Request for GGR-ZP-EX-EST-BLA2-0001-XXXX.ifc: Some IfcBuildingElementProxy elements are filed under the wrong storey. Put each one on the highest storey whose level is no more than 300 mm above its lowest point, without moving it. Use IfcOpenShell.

First a look at what the model holds.

```python
import ifcopenshell
import ifcopenshell.util.element
import ifcopenshell.util.placement

model = ifcopenshell.open("GGR-ZP-EX-EST-BLA2-0001-XXXX.ifc")
print(model.schema)
for storey in model.by_type("IfcBuildingStorey"):
    level = ifcopenshell.util.placement.get_storey_elevation(storey)
    count = sum(e.is_a("IfcBuildingElementProxy") for e in ifcopenshell.util.element.get_contained(storey))
    print(storey.id(), storey.Name, round(level, 3), count, sep=" | ")
```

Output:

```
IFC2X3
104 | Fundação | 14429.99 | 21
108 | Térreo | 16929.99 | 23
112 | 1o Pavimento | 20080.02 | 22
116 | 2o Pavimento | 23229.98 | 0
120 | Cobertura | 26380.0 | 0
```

```python
import ifcopenshell
import ifcopenshell.api.spatial
import ifcopenshell.geom
import ifcopenshell.util.element
import ifcopenshell.util.placement
import ifcopenshell.util.shape
import ifcopenshell.util.unit

model = ifcopenshell.open("GGR-ZP-EX-EST-BLA2-0001-XXXX.ifc")
unit_scale = ifcopenshell.util.unit.calculate_unit_scale(model)
settings = ifcopenshell.geom.settings()

levels = sorted(
    ((ifcopenshell.util.placement.get_storey_elevation(s) * unit_scale, s) for s in model.by_type("IfcBuildingStorey")),
    key=lambda pair: pair[0],
)

for e in model.by_type("IfcBuildingElementProxy"):
    current = e.ContainedInStructure[0].RelatingStructure if e.ContainedInStructure else None
    if current is None or not current.is_a("IfcBuildingStorey"):
        continue
    shape = ifcopenshell.geom.create_shape(settings, e)
    bottom = ifcopenshell.util.shape.get_shape_bottom_elevation(shape, shape.geometry)
    below = [s for level, s in levels if level <= bottom + 0.3]
    storey = below[-1] if below else levels[0][1]
    if storey != current:
        # assign_container keeps the world position.
        ifcopenshell.api.spatial.assign_container(model, products=[e], relating_structure=storey)
        print(e.id(), current.Name, "->", storey.Name)

model.write("GGR-ZP-EX-EST-BLA2-0001-XXXX_v2.ifc")
```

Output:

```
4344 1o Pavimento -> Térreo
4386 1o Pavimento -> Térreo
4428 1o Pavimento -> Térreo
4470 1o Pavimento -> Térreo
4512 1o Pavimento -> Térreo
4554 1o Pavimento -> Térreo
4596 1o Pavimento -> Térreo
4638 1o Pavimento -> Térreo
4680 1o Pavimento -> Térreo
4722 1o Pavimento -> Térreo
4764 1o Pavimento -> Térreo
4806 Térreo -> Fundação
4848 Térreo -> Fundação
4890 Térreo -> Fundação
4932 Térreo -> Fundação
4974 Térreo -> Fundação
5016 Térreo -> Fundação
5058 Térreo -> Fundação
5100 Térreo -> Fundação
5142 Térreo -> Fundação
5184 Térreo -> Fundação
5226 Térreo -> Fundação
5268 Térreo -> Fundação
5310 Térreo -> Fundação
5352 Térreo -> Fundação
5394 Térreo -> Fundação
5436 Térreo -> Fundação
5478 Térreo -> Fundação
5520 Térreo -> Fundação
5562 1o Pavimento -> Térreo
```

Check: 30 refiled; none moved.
